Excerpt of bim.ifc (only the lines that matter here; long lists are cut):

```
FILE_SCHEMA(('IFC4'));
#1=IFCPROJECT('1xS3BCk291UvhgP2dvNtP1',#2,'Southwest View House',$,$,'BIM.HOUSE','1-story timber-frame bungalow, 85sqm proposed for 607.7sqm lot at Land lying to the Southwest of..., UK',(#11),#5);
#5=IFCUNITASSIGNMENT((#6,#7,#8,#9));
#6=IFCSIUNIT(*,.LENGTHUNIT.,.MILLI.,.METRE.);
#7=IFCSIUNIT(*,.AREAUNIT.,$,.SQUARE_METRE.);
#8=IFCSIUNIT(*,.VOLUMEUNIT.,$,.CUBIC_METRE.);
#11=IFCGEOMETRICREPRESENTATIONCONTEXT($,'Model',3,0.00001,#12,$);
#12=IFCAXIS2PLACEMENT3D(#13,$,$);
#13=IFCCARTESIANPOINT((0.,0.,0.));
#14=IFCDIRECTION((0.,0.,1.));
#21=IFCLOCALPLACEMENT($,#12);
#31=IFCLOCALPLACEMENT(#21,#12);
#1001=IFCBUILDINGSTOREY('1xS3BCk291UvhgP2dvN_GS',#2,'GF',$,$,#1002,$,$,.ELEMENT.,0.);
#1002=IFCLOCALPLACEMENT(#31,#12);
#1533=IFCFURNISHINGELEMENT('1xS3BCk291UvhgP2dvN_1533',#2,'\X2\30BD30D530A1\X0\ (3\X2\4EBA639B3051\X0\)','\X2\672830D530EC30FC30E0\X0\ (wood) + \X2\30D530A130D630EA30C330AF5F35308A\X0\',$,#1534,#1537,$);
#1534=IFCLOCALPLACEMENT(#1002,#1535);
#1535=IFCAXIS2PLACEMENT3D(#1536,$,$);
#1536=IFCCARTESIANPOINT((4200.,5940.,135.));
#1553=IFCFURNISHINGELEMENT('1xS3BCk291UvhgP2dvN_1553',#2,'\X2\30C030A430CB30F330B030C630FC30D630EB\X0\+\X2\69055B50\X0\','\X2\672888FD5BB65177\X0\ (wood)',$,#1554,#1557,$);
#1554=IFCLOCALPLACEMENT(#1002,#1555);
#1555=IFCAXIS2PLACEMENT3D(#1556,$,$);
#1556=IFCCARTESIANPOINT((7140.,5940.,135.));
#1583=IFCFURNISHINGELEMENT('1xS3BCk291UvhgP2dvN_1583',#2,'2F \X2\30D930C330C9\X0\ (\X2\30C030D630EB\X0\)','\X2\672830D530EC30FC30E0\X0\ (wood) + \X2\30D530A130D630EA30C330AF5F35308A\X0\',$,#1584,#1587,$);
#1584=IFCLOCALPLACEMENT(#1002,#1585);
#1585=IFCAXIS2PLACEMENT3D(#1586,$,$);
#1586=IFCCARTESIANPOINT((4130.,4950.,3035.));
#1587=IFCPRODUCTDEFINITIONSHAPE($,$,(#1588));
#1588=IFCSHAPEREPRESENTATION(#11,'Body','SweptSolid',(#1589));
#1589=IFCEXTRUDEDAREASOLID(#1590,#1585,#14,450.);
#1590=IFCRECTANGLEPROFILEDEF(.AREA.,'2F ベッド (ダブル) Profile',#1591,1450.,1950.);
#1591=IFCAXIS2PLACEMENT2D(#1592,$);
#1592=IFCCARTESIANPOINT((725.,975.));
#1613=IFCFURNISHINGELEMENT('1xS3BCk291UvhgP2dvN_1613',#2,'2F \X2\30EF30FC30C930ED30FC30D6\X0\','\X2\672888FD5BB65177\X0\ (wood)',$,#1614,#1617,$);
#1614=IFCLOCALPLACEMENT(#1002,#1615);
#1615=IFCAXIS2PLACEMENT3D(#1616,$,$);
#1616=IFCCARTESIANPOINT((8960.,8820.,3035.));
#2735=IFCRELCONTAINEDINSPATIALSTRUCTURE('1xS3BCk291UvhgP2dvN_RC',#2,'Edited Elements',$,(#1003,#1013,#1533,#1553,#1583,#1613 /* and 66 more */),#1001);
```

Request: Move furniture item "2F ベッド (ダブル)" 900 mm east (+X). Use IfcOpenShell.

```python
import ifcopenshell
import ifcopenshell.api.geometry
import ifcopenshell.util.placement

model = ifcopenshell.open("bim.ifc")

item = model.by_id(1583)
matrix = ifcopenshell.util.placement.get_local_placement(item.ObjectPlacement)
matrix[0, 3] += 900.0
ifcopenshell.api.geometry.edit_object_placement(model, product=item, matrix=matrix, is_si=False)

print(ifcopenshell.util.placement.get_local_placement(item.ObjectPlacement).round(3) + 0.0)

model.write("bim_v2.ifc")
```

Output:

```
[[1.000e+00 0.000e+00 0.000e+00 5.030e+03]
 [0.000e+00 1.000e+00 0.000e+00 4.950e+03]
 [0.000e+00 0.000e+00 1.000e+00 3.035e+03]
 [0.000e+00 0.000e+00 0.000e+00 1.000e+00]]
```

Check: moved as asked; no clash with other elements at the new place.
